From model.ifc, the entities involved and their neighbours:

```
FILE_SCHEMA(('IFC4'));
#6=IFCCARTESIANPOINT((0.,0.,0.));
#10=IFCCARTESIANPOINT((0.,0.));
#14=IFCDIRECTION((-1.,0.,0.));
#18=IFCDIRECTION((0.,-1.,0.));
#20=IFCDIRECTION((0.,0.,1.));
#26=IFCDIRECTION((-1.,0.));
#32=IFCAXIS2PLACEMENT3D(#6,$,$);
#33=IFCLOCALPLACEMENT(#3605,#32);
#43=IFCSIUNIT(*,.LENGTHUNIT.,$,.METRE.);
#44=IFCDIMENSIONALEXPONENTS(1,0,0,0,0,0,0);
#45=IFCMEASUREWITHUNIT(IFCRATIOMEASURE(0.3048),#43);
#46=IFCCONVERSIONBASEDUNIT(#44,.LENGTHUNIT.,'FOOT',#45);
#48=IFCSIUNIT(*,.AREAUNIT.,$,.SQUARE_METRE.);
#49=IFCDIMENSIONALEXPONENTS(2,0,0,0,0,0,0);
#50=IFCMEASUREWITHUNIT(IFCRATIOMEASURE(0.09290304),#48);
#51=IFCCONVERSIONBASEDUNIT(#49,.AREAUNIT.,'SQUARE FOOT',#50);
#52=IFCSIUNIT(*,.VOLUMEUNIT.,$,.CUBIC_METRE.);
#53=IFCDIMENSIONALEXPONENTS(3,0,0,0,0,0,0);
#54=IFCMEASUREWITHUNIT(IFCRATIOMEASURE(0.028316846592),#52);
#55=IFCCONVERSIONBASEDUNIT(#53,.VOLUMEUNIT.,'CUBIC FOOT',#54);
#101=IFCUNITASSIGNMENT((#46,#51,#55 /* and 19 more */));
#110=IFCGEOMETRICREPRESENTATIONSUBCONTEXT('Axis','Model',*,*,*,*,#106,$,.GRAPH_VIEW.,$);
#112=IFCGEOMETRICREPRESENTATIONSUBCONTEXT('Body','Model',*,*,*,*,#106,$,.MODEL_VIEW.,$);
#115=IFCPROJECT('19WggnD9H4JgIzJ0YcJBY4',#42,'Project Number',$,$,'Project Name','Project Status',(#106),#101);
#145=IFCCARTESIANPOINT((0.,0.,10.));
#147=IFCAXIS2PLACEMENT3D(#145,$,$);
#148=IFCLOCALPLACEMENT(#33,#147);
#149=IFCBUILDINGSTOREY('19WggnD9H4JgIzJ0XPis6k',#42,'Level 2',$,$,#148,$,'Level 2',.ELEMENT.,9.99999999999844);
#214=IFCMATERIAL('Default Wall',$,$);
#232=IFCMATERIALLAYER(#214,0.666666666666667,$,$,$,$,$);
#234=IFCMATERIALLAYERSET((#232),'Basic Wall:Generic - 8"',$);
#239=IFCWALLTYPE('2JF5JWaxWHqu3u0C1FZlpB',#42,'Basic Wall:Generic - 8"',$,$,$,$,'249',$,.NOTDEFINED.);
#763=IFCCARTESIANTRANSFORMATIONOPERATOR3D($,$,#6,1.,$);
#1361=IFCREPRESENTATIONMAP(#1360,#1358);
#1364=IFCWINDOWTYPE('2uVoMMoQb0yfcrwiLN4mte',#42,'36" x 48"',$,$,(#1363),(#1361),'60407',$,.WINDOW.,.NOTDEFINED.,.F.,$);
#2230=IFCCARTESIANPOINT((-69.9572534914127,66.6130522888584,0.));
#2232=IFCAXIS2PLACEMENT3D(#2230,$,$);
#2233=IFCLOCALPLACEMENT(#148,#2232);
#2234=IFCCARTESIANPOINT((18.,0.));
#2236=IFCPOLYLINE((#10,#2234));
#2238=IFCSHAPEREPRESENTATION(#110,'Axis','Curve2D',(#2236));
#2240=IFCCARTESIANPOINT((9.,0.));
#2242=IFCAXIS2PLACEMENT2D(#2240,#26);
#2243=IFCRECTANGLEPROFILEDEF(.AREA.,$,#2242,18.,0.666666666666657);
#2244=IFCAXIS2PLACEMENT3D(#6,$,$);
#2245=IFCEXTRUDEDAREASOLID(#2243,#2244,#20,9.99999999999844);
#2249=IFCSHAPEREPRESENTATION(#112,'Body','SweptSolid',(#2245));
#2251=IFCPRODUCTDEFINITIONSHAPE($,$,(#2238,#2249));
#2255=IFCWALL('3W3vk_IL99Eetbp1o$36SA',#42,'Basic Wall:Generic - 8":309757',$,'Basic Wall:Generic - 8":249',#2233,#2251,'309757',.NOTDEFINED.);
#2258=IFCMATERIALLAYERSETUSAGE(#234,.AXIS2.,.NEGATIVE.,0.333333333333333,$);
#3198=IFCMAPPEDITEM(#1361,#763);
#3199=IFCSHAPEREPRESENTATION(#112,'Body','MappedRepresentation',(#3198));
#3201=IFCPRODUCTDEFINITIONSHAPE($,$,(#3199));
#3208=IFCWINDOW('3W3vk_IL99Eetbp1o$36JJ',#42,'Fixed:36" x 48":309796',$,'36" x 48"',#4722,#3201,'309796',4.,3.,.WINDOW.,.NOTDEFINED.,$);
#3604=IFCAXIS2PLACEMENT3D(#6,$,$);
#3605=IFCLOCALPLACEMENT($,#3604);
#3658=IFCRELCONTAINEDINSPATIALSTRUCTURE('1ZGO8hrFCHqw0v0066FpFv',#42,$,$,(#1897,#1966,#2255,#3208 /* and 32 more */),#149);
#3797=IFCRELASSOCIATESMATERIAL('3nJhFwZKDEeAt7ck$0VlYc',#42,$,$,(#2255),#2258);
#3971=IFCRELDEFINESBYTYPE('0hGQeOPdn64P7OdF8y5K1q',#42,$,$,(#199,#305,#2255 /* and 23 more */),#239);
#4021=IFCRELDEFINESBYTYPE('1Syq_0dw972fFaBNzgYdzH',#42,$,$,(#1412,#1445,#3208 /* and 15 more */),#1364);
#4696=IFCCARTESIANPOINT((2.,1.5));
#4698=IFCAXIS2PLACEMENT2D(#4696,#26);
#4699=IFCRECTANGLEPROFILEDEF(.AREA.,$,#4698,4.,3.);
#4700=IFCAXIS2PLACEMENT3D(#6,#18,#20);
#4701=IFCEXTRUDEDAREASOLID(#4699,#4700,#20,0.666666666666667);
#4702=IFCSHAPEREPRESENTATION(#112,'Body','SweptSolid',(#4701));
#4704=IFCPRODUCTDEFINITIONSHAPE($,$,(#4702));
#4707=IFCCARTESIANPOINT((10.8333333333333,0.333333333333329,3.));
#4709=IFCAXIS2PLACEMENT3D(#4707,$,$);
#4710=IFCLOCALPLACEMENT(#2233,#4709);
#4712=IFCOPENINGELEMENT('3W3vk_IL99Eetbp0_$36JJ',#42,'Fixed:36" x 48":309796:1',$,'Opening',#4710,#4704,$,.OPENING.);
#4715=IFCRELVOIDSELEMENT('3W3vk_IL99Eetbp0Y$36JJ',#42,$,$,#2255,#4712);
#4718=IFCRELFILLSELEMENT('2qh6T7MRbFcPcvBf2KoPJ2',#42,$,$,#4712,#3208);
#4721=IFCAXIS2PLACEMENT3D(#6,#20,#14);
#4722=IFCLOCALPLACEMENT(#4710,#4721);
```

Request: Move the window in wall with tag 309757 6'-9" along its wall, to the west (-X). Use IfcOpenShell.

```python
import ifcopenshell
import ifcopenshell.api.geometry
import ifcopenshell.util.placement
import ifcopenshell.util.unit

model = ifcopenshell.open("model.ifc")
unit_scale = ifcopenshell.util.unit.calculate_unit_scale(model)

window = model.by_guid("3W3vk_IL99Eetbp1o$36JJ")
opening = window.FillsVoids[0].RelatingOpeningElement
wall = opening.VoidsElements[0].RelatingBuildingElement

wall_matrix = ifcopenshell.util.placement.get_local_placement(wall.ObjectPlacement)
shift = wall_matrix[:3, 0] * -81 * 0.0254 / unit_scale
before = ifcopenshell.util.placement.get_local_placement(window.ObjectPlacement)[:3, 3].copy()

# The window is placed relative to its opening, so it follows when the opening moves.
matrix = ifcopenshell.util.placement.get_local_placement(opening.ObjectPlacement)
matrix[:3, 3] += shift
ifcopenshell.api.geometry.edit_object_placement(
    model, product=opening, matrix=matrix, is_si=False, should_transform_children=True
)

after = ifcopenshell.util.placement.get_local_placement(window.ObjectPlacement)[:3, 3]
print("window moved by", (after - before).round(3) + 0.0)

model.write("model_updated.ifc")
```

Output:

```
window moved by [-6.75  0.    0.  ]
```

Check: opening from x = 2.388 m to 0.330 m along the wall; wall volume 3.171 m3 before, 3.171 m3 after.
